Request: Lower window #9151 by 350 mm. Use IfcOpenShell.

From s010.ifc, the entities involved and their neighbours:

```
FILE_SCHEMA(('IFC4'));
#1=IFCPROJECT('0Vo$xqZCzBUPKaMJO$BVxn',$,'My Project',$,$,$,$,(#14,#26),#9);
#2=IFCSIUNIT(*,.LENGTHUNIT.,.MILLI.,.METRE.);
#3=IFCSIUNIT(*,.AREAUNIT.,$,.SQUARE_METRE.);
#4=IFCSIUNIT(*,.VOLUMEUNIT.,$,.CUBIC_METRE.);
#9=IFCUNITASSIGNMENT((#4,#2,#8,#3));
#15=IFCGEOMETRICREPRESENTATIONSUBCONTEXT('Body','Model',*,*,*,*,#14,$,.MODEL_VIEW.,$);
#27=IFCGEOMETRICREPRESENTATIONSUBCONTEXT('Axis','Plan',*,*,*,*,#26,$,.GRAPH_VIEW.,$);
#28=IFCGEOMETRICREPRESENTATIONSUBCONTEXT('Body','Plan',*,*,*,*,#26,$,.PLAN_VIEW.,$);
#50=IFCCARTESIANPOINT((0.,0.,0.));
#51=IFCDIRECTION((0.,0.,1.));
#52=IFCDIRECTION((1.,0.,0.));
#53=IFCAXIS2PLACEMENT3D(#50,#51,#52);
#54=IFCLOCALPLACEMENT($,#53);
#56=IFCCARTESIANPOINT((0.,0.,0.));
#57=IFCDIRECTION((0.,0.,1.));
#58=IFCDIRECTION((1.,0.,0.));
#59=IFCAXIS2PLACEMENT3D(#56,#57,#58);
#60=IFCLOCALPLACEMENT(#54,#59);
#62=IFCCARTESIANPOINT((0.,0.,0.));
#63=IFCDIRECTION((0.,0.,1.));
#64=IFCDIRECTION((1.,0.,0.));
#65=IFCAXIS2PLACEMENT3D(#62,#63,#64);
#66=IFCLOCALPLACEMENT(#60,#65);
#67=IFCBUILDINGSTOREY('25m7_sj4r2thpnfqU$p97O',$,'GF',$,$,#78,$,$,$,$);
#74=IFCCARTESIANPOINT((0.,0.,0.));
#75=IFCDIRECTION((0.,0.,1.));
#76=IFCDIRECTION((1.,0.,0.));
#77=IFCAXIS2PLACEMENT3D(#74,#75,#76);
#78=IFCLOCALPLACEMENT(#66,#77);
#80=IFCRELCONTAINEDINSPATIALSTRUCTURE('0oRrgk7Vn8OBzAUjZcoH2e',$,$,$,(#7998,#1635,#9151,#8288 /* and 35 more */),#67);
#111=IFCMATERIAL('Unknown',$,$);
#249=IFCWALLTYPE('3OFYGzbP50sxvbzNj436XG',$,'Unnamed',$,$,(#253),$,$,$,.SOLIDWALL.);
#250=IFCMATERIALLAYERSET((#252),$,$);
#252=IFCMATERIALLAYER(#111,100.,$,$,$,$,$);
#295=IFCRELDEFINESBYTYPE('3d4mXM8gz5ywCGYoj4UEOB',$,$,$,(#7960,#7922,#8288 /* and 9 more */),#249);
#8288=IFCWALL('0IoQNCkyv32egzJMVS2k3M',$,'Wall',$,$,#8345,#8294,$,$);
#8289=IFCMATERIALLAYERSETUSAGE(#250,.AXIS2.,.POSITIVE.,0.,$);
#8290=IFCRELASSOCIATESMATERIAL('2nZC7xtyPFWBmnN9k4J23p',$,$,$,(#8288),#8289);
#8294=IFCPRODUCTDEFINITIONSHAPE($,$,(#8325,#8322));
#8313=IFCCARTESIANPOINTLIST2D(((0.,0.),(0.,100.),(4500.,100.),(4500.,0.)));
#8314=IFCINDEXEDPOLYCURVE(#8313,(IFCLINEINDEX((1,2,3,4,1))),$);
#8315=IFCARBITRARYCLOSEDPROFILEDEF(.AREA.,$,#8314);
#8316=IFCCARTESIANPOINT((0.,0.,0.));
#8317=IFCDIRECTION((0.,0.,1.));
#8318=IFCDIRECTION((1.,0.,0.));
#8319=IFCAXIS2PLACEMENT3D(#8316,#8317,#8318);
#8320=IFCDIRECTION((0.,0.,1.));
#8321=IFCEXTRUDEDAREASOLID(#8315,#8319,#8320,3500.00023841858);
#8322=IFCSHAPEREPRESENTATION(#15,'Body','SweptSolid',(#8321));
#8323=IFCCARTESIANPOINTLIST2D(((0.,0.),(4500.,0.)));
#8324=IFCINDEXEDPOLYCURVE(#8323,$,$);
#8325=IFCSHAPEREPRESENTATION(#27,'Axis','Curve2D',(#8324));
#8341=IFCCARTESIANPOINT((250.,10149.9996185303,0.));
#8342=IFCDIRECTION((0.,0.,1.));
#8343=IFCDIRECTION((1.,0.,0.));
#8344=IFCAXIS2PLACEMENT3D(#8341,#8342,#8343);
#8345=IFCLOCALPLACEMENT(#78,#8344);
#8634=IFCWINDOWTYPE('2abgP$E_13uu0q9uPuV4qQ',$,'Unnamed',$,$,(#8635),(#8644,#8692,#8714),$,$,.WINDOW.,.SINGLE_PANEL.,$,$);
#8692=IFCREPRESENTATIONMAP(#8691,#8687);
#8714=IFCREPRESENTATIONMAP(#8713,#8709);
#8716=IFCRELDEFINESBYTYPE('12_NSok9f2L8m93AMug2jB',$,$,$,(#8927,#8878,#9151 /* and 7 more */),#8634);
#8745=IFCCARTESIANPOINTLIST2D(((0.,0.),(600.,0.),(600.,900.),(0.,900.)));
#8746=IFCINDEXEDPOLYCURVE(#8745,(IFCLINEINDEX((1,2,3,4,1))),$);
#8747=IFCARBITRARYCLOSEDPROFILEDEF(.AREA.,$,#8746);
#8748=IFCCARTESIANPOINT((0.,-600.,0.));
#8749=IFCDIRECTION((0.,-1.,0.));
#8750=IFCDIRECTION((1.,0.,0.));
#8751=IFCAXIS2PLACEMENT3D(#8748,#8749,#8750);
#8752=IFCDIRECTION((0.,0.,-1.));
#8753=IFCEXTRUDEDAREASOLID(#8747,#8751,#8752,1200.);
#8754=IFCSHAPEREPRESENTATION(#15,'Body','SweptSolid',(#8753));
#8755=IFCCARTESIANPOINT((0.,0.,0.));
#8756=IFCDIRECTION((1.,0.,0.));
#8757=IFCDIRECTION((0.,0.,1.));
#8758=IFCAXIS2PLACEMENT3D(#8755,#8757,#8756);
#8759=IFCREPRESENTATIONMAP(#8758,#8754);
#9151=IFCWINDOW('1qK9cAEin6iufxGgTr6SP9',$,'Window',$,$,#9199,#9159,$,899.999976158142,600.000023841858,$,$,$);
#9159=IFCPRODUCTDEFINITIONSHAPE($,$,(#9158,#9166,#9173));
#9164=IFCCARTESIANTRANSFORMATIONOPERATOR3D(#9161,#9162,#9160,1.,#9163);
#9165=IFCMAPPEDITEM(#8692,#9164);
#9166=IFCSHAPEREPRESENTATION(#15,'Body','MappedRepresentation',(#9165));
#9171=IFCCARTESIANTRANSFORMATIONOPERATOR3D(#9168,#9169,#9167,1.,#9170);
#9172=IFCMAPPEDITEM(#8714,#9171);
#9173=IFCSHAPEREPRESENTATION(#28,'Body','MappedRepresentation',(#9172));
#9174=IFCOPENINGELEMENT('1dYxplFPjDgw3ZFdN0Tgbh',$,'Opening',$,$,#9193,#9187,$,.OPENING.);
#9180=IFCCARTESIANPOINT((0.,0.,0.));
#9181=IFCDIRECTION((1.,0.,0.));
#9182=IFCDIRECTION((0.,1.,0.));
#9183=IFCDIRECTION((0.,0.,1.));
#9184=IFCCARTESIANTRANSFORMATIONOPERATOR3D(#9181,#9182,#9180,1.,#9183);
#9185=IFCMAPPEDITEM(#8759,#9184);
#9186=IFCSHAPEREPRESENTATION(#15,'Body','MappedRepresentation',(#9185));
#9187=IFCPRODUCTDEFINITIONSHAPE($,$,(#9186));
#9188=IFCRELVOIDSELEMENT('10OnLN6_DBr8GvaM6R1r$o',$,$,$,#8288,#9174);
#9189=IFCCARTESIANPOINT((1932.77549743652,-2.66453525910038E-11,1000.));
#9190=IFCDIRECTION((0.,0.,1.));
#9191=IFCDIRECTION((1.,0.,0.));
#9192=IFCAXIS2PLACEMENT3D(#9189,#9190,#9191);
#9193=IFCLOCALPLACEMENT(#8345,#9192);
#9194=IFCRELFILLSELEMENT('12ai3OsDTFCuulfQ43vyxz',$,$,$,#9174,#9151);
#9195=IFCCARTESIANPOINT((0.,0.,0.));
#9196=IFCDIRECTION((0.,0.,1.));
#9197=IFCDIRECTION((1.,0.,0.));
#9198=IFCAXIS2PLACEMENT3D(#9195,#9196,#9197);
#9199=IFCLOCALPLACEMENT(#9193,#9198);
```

```python
import numpy as np
import ifcopenshell
import ifcopenshell.api.geometry
import ifcopenshell.util.placement
import ifcopenshell.util.unit

model = ifcopenshell.open("s010.ifc")
unit_scale = ifcopenshell.util.unit.calculate_unit_scale(model)

window = model.by_guid("1qK9cAEin6iufxGgTr6SP9")
opening = window.FillsVoids[0].RelatingOpeningElement
dz = -350.0

shift = np.array([0.0, 0.0, dz])
# The window is placed relative to its opening, so it follows when the opening moves.
matrix = ifcopenshell.util.placement.get_local_placement(opening.ObjectPlacement)
matrix[:3, 3] += shift
ifcopenshell.api.geometry.edit_object_placement(
    model, product=opening, matrix=matrix, is_si=False, should_transform_children=True
)

print(f"moved by {dz * unit_scale:+.3f} m")

model.write("s010_edited.ifc")
```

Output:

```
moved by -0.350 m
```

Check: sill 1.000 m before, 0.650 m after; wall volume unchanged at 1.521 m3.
